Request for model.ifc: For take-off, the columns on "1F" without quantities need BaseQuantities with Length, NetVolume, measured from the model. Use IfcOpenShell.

First a look at what the model holds.

```python
import ifcopenshell
import ifcopenshell.util.element
import ifcopenshell.util.unit

model = ifcopenshell.open("model.ifc")
print(model.schema)
for unit_type in ("LENGTHUNIT", "AREAUNIT", "VOLUMEUNIT"):
    print(unit_type, ifcopenshell.util.unit.calculate_unit_scale(model, unit_type))
storey = next(s for s in model.by_type("IfcBuildingStorey") if s.Name == "1F")
columns = [e for e in ifcopenshell.util.element.get_decomposition(storey) if e.is_a("IfcColumn")]
for e in sorted(columns, key=lambda e: e.id()):
    print(e.id(), e.is_a(), e.Name, list(ifcopenshell.util.element.get_psets(e, qtos_only=True)), sep=" | ")
```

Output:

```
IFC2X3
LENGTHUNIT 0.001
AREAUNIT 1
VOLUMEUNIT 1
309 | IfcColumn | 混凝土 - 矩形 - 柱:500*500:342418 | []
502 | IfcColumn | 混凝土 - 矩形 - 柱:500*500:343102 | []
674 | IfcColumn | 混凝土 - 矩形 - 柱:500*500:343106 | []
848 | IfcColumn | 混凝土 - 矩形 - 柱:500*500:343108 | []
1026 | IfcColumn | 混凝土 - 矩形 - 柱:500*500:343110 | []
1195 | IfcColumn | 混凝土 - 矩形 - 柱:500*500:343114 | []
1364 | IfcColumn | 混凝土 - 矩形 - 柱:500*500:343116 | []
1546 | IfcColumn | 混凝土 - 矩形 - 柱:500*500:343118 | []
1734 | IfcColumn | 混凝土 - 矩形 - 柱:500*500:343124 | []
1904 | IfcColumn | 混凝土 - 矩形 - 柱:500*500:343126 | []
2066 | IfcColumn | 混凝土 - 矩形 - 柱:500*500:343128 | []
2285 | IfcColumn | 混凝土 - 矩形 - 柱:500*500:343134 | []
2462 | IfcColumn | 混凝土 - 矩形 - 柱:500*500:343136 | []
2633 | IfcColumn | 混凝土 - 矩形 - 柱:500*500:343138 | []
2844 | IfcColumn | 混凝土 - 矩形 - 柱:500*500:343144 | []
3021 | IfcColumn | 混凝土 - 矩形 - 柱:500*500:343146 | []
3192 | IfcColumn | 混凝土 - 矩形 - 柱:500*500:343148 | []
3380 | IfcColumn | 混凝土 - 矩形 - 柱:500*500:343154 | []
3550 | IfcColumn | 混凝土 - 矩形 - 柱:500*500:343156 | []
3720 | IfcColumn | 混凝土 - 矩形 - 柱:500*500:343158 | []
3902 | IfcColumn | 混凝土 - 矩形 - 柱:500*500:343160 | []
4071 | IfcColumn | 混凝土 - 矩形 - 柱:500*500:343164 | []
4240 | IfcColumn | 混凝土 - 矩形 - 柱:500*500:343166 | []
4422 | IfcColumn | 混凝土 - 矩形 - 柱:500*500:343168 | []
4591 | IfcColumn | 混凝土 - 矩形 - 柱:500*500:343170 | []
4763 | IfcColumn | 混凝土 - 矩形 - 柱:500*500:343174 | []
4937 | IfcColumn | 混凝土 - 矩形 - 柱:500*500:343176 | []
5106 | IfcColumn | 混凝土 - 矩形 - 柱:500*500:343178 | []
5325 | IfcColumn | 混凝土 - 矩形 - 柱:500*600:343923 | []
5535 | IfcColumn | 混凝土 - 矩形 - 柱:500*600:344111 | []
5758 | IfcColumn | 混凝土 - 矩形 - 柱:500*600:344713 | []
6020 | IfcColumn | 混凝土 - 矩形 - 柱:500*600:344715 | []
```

```python
import ifcopenshell
import ifcopenshell.api.pset
import ifcopenshell.geom
import ifcopenshell.util.element
import ifcopenshell.util.shape
import ifcopenshell.util.unit

model = ifcopenshell.open("model.ifc")
unit_scale = ifcopenshell.util.unit.calculate_unit_scale(model)
volume_scale = ifcopenshell.util.unit.calculate_unit_scale(model, "VOLUMEUNIT")
settings = ifcopenshell.geom.settings()

storey = next(s for s in model.by_type("IfcBuildingStorey") if s.Name == "1F")
columns = [e for e in ifcopenshell.util.element.get_decomposition(storey) if e.is_a("IfcColumn")]

for e in sorted(columns, key=lambda e: e.id()):
    if ifcopenshell.util.element.get_psets(e, qtos_only=True, should_inherit=False):
        continue
    # Geometry comes back in metres, in the element's own axes.
    shape = ifcopenshell.geom.create_shape(settings, e)
    values = {
        "Length": ifcopenshell.util.shape.get_z(shape.geometry) / unit_scale,
        "NetVolume": ifcopenshell.util.shape.get_volume(shape.geometry) / volume_scale,
    }
    qto = ifcopenshell.api.pset.add_qto(model, product=e, name="BaseQuantities")
    ifcopenshell.api.pset.edit_qto(model, qto=qto, properties=values)
    print(e.id(), {k: round(v, 3) for k, v in values.items()})

model.write("model_rev.ifc")
```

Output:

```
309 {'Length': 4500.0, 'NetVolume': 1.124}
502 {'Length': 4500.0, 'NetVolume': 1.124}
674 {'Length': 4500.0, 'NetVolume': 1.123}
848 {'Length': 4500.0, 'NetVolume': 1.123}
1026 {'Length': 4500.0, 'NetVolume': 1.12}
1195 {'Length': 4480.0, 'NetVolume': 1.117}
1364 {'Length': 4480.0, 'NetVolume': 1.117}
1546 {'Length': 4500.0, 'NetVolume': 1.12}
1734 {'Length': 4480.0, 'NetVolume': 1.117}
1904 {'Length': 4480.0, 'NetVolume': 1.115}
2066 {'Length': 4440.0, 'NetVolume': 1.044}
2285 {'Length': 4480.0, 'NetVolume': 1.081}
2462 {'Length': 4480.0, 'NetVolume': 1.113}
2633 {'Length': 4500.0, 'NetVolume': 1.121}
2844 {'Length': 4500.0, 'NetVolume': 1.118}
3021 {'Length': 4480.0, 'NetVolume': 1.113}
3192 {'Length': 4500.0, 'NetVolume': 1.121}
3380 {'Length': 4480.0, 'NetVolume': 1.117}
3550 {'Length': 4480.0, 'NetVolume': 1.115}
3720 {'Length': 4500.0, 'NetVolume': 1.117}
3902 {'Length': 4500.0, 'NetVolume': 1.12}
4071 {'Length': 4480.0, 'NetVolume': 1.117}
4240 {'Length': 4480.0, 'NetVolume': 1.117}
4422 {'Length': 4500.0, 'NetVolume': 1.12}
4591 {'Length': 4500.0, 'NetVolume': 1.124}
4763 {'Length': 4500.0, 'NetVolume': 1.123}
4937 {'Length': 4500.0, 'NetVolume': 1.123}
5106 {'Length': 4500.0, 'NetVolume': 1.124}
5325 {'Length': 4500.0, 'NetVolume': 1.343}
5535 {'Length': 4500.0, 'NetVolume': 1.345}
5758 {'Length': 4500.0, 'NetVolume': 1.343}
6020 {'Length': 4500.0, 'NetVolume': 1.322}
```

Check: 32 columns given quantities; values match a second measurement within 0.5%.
